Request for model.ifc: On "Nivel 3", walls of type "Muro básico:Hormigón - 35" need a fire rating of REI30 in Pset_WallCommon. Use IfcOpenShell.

First a look at what the model holds.

```python
import ifcopenshell
import ifcopenshell.util.element

model = ifcopenshell.open("model.ifc")
print(model.schema)
storey = next(s for s in model.by_type("IfcBuildingStorey") if s.Name == "Nivel 3")
walls = [e for e in ifcopenshell.util.element.get_decomposition(storey) if e.is_a("IfcWall")]
seen = {}
for e in walls:
    element_type = ifcopenshell.util.element.get_type(e)
    key = (element_type.Name if element_type != e and element_type else None, ifcopenshell.util.element.get_pset(e, "Pset_WallCommon", "FireRating"))
    seen[key] = seen.get(key, 0) + 1
for (name, value), count in sorted(seen.items(), key=str):
    print(count, "x", name, "|", value)
```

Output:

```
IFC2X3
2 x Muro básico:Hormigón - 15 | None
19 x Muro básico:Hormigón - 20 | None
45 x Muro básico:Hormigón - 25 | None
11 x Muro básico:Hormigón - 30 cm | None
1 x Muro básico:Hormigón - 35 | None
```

```python
import ifcopenshell
import ifcopenshell.api.pset
import ifcopenshell.util.element

model = ifcopenshell.open("model.ifc")

storey = next(s for s in model.by_type("IfcBuildingStorey") if s.Name == "Nivel 3")
walls = [e for e in ifcopenshell.util.element.get_decomposition(storey) if e.is_a("IfcWall")]

count = 0
for e in walls:
    element_type = ifcopenshell.util.element.get_type(e)
    if element_type in (None, e) or element_type.Name != "Muro básico:Hormigón - 35":
        continue
    # add_pset returns the element's existing set when there is one.
    pset = ifcopenshell.api.pset.add_pset(model, product=e, name="Pset_WallCommon")
    ifcopenshell.api.pset.edit_pset(model, pset=pset, properties={"FireRating": "REI30"})
    count += 1

print(count, "walls updated")

model.write("model_rev.ifc")
```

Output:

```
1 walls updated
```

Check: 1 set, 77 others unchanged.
